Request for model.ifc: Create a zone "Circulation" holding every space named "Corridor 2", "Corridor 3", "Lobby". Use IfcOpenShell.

First a look at what the model holds.

```python
import ifcopenshell

model = ifcopenshell.open("model.ifc")
print(model.schema)
seen = {}
for space in model.by_type("IfcSpace"):
    seen[space.Name] = seen.get(space.Name, 0) + 1
for name, count in sorted(seen.items(), key=str):
    print(count, "x", name)
print("zones:", [z.Name for z in model.by_type("IfcZone")][:20])
```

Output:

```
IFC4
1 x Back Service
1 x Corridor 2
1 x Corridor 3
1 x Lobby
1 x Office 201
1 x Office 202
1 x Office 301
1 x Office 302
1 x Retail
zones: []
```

```python
import ifcopenshell
import ifcopenshell.api.group
import ifcopenshell.api.root

model = ifcopenshell.open("model.ifc")

names = {"Corridor 2", "Corridor 3", "Lobby"}
spaces = [s for s in model.by_type("IfcSpace") if s.Name in names]

zone = ifcopenshell.api.root.create_entity(model, ifc_class="IfcZone", name="Circulation")
ifcopenshell.api.group.assign_group(model, products=spaces, group=zone)
print(len(spaces), "spaces in", zone.Name)

model.write("model_updated.ifc")
```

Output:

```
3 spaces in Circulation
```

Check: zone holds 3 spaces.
